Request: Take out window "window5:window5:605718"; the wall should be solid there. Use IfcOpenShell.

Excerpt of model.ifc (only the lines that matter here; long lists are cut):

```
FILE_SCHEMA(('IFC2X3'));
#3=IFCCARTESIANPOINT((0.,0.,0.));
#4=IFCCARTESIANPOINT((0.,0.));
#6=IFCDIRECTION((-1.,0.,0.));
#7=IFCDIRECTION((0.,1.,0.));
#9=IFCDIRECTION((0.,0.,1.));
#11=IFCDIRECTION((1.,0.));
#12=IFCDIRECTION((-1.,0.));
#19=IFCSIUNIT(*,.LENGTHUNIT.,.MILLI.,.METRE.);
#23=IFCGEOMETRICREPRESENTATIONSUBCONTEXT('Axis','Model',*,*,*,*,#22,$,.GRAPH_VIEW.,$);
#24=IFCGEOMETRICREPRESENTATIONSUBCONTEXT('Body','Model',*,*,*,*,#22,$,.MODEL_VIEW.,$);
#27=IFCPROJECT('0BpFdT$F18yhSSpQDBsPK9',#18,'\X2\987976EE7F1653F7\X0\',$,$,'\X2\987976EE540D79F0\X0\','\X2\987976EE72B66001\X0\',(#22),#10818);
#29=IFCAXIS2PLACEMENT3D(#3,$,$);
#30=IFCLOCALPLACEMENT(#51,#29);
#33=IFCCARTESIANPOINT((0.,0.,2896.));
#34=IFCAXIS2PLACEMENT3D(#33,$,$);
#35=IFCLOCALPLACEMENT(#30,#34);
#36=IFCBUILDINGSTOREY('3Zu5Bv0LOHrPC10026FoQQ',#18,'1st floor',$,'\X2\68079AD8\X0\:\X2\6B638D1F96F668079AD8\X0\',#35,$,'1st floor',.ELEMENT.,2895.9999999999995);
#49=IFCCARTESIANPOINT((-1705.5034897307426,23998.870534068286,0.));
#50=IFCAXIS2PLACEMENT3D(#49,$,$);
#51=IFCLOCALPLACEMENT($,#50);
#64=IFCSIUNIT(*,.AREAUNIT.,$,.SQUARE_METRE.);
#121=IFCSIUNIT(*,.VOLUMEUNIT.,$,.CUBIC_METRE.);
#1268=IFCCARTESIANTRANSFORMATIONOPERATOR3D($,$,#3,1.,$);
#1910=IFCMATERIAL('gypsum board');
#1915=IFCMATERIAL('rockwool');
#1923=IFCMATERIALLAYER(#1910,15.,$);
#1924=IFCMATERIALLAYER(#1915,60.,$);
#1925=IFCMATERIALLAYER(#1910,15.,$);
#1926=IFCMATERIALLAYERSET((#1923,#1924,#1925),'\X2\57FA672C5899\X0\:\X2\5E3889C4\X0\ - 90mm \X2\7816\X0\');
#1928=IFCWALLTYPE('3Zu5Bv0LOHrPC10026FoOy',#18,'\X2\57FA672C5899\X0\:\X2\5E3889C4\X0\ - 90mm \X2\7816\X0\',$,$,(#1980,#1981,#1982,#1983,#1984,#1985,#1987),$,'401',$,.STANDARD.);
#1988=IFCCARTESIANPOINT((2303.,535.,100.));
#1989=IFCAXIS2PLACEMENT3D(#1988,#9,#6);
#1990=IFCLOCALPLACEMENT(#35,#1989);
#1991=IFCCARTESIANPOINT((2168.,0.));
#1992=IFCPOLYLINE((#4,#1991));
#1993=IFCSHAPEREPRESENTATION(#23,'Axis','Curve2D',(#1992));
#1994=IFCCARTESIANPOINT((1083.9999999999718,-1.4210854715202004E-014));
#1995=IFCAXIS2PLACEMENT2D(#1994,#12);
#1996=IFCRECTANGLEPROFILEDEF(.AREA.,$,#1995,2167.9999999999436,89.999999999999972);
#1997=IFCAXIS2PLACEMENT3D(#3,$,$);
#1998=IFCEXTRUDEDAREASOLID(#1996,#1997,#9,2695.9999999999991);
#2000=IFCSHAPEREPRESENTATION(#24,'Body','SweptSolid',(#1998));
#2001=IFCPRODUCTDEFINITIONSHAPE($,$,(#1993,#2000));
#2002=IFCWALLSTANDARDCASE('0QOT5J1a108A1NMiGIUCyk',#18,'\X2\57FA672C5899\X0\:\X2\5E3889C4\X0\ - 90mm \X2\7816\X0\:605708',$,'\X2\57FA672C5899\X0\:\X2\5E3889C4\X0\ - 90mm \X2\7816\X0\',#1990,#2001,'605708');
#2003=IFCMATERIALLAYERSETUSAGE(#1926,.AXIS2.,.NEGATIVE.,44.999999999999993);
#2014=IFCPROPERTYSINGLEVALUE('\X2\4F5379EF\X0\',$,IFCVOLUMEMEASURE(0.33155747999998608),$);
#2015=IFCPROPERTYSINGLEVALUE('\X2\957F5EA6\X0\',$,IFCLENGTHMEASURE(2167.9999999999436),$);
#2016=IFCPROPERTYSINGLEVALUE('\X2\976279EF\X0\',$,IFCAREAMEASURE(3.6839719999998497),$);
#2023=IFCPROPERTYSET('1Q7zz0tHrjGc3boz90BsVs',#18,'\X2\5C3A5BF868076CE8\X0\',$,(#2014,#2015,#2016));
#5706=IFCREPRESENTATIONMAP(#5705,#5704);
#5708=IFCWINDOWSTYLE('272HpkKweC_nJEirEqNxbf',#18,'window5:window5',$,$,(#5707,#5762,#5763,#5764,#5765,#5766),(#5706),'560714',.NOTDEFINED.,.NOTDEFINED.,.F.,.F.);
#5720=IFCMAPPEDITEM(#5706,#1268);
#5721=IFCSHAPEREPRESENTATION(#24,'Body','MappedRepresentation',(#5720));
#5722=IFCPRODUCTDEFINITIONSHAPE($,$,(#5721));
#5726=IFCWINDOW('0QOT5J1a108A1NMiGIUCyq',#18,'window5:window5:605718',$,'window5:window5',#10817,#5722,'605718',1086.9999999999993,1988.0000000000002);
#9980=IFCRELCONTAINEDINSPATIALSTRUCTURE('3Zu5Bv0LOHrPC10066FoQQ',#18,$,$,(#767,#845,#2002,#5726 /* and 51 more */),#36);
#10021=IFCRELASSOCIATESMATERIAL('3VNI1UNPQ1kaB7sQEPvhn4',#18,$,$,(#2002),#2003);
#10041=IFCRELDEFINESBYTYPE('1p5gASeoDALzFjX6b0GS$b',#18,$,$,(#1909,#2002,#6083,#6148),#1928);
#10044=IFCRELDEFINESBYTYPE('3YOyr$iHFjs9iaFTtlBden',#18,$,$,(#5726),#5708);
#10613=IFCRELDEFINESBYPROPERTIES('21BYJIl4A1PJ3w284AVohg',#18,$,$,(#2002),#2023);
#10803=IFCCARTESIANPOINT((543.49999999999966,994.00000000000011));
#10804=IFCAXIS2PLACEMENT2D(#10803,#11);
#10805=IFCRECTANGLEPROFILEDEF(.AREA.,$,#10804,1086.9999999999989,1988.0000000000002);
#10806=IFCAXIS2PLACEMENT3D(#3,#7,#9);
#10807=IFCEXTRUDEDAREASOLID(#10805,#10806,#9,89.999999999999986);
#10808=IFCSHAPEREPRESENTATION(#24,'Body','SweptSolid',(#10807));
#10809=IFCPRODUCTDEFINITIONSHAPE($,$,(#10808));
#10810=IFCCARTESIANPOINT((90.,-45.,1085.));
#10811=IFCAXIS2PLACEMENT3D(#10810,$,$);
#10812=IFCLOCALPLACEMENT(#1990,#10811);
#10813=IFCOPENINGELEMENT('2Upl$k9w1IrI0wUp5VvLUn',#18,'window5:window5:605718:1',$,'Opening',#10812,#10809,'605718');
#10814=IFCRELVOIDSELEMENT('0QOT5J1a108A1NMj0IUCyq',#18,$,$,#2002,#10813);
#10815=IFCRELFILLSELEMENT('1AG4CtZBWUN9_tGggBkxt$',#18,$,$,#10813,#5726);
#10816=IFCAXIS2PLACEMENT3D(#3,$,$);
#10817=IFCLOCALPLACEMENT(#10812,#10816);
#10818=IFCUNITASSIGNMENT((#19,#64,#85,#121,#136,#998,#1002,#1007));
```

```python
import ifcopenshell
import ifcopenshell.api.feature
import ifcopenshell.api.pset
import ifcopenshell.api.root
import ifcopenshell.geom
import ifcopenshell.util.element
import ifcopenshell.util.shape
import ifcopenshell.util.unit

model = ifcopenshell.open("model.ifc")
area_scale = ifcopenshell.util.unit.calculate_unit_scale(model, "AREAUNIT")
volume_scale = ifcopenshell.util.unit.calculate_unit_scale(model, "VOLUMEUNIT")
settings = ifcopenshell.geom.settings()


def volume(element):
    """Net volume in cubic metres, openings subtracted."""
    shape = ifcopenshell.geom.create_shape(settings, element)
    return ifcopenshell.util.shape.get_volume(shape.geometry)


window = model.by_guid("0QOT5J1a108A1NMiGIUCyq")
opening = window.FillsVoids[0].RelatingOpeningElement
wall = opening.VoidsElements[0].RelatingBuildingElement
before = volume(wall)

ifcopenshell.api.root.remove_product(model, product=window)
ifcopenshell.api.feature.remove_feature(model, feature=opening)

after = volume(wall)
thickness = 0.09  # wall thickness in metres

# Update the wall's stored quantities.
pset = model.by_id(ifcopenshell.util.element.get_pset(wall, "尺寸标注", should_inherit=False)["id"])
ifcopenshell.api.pset.edit_pset(model, pset=pset, properties={
    "体积": model.create_entity("IfcVolumeMeasure", after / volume_scale),
    "面积": model.create_entity("IfcAreaMeasure", after / thickness / area_scale),
})

print(f"wall volume {before:.3f} -> {after:.3f} m3")

model.write("model_edited.ifc")
```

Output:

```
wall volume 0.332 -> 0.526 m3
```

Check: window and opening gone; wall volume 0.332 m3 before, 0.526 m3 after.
